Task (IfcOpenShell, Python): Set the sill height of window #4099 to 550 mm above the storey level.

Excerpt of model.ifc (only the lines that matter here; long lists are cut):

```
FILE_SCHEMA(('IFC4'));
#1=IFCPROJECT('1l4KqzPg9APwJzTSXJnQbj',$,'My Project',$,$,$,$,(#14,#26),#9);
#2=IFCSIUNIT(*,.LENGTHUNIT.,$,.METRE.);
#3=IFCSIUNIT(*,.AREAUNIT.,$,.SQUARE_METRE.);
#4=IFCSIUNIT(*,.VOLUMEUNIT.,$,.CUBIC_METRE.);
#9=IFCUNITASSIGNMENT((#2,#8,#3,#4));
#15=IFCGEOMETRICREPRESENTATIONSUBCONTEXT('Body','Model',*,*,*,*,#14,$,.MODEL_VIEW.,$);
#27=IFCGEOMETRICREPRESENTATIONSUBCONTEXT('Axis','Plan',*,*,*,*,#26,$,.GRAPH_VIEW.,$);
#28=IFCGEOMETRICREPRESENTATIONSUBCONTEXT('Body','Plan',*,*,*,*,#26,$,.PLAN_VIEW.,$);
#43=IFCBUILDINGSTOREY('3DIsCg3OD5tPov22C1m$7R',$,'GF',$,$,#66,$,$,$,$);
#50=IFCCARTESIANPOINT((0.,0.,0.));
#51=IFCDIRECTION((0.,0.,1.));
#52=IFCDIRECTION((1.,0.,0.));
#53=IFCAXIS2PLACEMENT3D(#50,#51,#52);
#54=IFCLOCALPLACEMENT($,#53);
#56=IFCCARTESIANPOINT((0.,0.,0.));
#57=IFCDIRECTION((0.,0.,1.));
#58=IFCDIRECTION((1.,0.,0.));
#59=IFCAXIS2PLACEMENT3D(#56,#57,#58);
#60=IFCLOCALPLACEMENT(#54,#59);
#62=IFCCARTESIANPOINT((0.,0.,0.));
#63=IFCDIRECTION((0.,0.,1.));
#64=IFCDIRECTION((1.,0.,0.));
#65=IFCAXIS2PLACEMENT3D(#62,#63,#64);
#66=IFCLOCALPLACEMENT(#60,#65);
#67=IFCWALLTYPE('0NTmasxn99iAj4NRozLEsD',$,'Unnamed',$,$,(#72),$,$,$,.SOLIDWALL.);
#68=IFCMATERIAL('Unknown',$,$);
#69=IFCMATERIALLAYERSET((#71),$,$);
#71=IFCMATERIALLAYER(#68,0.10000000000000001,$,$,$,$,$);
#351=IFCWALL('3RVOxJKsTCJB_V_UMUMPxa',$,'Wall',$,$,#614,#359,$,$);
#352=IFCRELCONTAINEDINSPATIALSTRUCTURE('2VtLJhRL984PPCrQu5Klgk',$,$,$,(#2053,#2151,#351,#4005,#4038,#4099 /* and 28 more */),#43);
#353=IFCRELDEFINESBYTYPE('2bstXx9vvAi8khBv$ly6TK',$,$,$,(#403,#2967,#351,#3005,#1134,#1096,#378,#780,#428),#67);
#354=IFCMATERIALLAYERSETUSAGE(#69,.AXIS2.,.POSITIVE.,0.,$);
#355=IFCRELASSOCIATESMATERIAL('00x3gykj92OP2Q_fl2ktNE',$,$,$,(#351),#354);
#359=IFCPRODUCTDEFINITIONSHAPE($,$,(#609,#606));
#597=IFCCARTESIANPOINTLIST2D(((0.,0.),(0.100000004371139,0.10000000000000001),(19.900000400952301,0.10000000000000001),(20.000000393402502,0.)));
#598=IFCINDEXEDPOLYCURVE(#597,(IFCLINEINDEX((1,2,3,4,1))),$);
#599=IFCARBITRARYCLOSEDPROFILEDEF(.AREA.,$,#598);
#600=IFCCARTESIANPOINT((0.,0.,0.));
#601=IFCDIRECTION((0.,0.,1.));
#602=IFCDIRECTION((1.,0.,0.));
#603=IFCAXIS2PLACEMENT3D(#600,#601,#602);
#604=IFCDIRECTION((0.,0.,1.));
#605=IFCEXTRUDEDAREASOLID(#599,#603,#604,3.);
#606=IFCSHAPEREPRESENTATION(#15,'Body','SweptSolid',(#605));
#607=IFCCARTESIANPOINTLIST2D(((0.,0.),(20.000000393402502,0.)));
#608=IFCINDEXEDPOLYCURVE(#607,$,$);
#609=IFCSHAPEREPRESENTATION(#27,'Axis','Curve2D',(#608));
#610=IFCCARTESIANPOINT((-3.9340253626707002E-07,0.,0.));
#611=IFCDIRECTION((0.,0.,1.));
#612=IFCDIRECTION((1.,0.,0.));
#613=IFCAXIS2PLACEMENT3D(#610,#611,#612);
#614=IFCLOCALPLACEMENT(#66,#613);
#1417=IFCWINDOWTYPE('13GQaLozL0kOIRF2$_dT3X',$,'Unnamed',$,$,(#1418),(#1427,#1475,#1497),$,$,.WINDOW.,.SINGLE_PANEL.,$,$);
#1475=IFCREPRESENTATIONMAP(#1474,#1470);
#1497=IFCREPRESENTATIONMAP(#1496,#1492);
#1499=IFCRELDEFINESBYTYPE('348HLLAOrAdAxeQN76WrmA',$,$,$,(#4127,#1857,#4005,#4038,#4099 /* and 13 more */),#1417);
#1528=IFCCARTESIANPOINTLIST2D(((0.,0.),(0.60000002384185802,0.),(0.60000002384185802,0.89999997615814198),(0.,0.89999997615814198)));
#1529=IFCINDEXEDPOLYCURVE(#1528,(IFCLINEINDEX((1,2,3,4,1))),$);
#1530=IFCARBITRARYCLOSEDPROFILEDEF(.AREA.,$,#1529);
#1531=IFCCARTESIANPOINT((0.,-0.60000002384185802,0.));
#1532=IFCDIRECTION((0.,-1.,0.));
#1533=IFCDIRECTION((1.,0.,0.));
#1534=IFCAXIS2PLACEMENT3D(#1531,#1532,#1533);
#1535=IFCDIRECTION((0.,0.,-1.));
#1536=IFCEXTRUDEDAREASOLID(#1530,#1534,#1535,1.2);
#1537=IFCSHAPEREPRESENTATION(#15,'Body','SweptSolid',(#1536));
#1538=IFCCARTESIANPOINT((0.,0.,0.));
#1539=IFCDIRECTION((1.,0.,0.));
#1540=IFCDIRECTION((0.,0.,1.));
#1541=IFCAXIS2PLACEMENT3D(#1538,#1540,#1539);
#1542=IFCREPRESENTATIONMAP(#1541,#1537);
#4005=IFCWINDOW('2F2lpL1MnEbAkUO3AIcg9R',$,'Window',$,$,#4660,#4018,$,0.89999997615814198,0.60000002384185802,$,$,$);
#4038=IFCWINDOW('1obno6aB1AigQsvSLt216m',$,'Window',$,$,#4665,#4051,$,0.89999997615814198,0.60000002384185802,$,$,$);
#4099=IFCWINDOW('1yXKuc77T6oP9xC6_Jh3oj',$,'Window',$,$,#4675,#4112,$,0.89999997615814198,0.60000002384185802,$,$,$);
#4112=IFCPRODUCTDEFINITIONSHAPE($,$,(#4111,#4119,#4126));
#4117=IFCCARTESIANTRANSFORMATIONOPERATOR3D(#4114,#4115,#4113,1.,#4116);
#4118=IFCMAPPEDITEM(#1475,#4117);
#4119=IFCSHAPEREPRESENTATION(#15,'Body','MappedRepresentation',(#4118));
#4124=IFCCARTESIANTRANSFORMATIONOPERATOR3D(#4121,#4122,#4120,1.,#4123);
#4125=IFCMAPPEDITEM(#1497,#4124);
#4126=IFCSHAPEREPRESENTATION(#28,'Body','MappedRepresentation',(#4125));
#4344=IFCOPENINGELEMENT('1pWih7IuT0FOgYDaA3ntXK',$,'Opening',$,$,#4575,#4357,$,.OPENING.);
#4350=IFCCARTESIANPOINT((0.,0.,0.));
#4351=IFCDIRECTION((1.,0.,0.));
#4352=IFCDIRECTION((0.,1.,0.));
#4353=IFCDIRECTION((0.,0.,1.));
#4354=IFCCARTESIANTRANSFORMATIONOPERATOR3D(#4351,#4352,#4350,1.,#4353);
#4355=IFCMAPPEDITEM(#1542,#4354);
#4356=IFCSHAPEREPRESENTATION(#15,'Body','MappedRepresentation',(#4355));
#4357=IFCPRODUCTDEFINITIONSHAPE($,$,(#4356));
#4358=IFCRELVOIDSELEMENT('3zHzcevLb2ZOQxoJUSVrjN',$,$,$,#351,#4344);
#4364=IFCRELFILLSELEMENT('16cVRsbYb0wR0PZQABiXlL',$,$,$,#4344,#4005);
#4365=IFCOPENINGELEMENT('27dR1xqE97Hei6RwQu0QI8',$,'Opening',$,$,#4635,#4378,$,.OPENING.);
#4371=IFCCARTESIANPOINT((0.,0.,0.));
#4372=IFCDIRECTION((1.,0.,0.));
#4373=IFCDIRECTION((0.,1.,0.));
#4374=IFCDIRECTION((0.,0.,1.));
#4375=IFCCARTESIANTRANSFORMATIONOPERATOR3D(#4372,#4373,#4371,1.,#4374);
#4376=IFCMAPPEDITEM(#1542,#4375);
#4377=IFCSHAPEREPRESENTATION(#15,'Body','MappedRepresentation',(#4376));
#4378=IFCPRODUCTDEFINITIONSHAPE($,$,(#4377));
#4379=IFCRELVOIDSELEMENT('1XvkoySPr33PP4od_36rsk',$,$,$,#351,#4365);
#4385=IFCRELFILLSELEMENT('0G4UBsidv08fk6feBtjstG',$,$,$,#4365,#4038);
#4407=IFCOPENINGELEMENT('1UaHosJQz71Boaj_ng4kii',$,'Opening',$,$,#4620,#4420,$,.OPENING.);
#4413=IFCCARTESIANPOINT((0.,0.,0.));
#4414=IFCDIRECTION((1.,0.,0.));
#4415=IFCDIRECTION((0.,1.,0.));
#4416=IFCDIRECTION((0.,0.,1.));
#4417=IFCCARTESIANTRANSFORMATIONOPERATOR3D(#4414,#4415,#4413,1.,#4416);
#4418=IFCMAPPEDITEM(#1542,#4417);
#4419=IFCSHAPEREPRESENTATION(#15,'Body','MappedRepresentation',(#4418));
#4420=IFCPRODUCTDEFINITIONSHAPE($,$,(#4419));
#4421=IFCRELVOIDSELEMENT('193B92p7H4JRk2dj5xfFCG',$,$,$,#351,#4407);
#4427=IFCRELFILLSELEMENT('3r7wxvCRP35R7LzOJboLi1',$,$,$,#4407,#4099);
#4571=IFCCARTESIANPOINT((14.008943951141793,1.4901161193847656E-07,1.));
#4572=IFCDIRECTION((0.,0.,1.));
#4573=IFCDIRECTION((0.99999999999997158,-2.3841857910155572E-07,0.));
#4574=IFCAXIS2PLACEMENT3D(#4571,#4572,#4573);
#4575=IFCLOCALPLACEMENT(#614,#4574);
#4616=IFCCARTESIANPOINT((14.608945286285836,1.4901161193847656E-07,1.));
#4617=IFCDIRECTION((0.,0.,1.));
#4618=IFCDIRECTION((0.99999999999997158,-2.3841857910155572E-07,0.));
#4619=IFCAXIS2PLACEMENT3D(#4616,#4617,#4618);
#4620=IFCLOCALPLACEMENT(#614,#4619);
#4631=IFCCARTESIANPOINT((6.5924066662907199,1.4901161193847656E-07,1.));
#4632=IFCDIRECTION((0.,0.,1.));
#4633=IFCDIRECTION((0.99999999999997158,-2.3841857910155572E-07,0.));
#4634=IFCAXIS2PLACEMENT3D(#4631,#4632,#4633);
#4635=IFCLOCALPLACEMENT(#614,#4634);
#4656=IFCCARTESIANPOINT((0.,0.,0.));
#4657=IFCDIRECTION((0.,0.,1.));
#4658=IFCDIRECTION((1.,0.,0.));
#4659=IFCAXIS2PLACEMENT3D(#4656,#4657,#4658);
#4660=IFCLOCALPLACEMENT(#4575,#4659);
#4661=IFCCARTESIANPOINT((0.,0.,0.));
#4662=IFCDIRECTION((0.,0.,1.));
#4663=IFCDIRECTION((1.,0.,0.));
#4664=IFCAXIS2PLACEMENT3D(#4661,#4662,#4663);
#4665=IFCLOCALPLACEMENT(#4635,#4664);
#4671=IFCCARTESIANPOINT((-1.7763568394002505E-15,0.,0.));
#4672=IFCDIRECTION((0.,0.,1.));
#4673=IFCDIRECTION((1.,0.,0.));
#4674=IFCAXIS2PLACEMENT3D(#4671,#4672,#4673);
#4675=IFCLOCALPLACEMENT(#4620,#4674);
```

```python
import numpy as np
import ifcopenshell
import ifcopenshell.api.geometry
import ifcopenshell.geom
import ifcopenshell.util.element
import ifcopenshell.util.placement
import ifcopenshell.util.shape
import ifcopenshell.util.unit

model = ifcopenshell.open("model.ifc")
unit_scale = ifcopenshell.util.unit.calculate_unit_scale(model)

window = model.by_guid("1yXKuc77T6oP9xC6_Jh3oj")
opening = window.FillsVoids[0].RelatingOpeningElement
storey = ifcopenshell.util.element.get_container(window, ifc_class="IfcBuildingStorey")
level = ifcopenshell.util.placement.get_local_placement(storey.ObjectPlacement)[2, 3]

# The opening's origin need not be at the sill, so measure its lowest point.
shape = ifcopenshell.geom.create_shape(ifcopenshell.geom.settings(), opening)
bottom = ifcopenshell.util.shape.get_shape_bottom_elevation(shape, shape.geometry) / unit_scale
dz = level + 0.55 - bottom

shift = np.array([0.0, 0.0, dz])
# The window is placed relative to its opening, so it follows when the opening moves.
matrix = ifcopenshell.util.placement.get_local_placement(opening.ObjectPlacement)
matrix[:3, 3] += shift
ifcopenshell.api.geometry.edit_object_placement(
    model, product=opening, matrix=matrix, is_si=False, should_transform_children=True
)

print(f"moved by {dz * unit_scale:+.3f} m")

model.write("model_rev.ifc")
```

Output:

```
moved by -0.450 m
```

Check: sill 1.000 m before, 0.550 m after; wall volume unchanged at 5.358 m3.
